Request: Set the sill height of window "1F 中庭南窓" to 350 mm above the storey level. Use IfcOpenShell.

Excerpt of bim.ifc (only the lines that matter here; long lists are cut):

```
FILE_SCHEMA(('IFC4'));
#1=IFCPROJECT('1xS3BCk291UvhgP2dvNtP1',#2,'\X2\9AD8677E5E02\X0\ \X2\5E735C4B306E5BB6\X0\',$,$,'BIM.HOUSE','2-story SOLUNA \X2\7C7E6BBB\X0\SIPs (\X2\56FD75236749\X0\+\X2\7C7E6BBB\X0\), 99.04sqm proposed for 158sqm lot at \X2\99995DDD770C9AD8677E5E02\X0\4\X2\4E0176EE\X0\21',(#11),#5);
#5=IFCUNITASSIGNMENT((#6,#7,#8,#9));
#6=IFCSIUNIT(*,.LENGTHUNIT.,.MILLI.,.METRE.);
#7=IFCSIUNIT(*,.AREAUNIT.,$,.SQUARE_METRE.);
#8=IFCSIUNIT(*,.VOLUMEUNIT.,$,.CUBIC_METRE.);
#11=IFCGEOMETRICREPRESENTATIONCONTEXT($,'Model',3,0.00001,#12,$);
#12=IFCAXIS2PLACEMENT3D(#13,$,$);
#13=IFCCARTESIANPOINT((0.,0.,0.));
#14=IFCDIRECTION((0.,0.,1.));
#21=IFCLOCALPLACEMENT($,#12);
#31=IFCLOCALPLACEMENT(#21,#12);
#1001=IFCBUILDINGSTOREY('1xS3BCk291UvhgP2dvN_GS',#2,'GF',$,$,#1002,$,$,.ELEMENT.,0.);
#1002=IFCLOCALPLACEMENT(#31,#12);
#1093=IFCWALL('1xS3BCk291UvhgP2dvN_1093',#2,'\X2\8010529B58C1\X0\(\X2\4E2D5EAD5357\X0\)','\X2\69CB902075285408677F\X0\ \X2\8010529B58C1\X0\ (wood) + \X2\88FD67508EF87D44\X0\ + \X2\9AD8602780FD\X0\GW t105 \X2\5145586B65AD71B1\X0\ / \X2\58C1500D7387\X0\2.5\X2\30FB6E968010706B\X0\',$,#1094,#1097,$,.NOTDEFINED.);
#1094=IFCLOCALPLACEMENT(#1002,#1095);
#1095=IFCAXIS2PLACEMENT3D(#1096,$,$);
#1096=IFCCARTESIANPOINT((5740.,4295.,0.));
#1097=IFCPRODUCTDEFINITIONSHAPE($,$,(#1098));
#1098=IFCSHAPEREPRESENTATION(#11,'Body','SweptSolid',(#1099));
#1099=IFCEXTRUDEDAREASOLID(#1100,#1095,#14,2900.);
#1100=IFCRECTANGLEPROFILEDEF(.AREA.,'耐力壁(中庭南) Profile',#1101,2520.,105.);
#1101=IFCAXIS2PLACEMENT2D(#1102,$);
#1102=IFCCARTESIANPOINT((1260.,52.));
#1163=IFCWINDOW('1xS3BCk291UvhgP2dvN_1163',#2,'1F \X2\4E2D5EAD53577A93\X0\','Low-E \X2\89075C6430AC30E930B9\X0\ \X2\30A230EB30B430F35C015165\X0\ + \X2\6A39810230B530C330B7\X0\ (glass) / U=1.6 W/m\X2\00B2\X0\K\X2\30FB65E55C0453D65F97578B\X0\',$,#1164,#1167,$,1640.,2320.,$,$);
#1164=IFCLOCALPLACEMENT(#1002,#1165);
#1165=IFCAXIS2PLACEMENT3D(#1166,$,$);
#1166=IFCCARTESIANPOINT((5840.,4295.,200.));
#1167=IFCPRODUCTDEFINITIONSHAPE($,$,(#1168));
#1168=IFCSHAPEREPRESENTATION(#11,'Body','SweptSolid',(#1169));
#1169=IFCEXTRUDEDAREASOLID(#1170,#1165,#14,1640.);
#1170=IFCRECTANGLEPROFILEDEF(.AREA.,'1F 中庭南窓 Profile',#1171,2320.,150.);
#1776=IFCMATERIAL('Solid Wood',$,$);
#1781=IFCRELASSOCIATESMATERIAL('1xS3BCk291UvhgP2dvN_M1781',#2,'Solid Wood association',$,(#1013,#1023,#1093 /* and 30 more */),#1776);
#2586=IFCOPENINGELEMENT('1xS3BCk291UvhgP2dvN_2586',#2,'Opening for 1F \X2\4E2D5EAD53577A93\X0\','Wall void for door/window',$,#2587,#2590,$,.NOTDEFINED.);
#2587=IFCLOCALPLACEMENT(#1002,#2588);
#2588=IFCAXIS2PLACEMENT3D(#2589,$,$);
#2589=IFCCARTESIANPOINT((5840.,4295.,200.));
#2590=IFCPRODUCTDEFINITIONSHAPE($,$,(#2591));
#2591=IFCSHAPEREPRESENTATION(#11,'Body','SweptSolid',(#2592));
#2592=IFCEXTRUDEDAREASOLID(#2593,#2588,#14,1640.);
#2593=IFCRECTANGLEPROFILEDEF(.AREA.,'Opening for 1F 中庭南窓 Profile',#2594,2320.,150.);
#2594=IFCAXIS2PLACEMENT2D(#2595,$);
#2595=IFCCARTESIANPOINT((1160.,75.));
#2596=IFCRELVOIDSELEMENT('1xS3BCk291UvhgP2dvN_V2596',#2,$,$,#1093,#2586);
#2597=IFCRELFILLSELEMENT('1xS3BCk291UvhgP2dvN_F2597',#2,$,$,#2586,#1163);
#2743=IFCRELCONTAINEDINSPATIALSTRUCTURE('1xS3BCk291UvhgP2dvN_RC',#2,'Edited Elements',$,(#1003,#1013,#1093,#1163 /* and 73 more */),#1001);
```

```python
import numpy as np
import ifcopenshell
import ifcopenshell.api.geometry
import ifcopenshell.geom
import ifcopenshell.util.element
import ifcopenshell.util.placement
import ifcopenshell.util.shape
import ifcopenshell.util.unit

model = ifcopenshell.open("bim.ifc")
unit_scale = ifcopenshell.util.unit.calculate_unit_scale(model)

window = model.by_guid("1xS3BCk291UvhgP2dvN_1163")
opening = window.FillsVoids[0].RelatingOpeningElement
storey = ifcopenshell.util.element.get_container(window, ifc_class="IfcBuildingStorey")
level = ifcopenshell.util.placement.get_local_placement(storey.ObjectPlacement)[2, 3]

# The opening's origin need not be at the sill, so measure its lowest point.
shape = ifcopenshell.geom.create_shape(ifcopenshell.geom.settings(), opening)
bottom = ifcopenshell.util.shape.get_shape_bottom_elevation(shape, shape.geometry) / unit_scale
dz = level + 350.0 - bottom

shift = np.array([0.0, 0.0, dz])
# The window is not placed relative to its opening, so move both.
for product in (opening, window):
    matrix = ifcopenshell.util.placement.get_local_placement(product.ObjectPlacement)
    matrix[:3, 3] += shift
    ifcopenshell.api.geometry.edit_object_placement(model, product=product, matrix=matrix, is_si=False)

print(f"moved by {dz * unit_scale:+.3f} m")

model.write("bim_edited.ifc")
```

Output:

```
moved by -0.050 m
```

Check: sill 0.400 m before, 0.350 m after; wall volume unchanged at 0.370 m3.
